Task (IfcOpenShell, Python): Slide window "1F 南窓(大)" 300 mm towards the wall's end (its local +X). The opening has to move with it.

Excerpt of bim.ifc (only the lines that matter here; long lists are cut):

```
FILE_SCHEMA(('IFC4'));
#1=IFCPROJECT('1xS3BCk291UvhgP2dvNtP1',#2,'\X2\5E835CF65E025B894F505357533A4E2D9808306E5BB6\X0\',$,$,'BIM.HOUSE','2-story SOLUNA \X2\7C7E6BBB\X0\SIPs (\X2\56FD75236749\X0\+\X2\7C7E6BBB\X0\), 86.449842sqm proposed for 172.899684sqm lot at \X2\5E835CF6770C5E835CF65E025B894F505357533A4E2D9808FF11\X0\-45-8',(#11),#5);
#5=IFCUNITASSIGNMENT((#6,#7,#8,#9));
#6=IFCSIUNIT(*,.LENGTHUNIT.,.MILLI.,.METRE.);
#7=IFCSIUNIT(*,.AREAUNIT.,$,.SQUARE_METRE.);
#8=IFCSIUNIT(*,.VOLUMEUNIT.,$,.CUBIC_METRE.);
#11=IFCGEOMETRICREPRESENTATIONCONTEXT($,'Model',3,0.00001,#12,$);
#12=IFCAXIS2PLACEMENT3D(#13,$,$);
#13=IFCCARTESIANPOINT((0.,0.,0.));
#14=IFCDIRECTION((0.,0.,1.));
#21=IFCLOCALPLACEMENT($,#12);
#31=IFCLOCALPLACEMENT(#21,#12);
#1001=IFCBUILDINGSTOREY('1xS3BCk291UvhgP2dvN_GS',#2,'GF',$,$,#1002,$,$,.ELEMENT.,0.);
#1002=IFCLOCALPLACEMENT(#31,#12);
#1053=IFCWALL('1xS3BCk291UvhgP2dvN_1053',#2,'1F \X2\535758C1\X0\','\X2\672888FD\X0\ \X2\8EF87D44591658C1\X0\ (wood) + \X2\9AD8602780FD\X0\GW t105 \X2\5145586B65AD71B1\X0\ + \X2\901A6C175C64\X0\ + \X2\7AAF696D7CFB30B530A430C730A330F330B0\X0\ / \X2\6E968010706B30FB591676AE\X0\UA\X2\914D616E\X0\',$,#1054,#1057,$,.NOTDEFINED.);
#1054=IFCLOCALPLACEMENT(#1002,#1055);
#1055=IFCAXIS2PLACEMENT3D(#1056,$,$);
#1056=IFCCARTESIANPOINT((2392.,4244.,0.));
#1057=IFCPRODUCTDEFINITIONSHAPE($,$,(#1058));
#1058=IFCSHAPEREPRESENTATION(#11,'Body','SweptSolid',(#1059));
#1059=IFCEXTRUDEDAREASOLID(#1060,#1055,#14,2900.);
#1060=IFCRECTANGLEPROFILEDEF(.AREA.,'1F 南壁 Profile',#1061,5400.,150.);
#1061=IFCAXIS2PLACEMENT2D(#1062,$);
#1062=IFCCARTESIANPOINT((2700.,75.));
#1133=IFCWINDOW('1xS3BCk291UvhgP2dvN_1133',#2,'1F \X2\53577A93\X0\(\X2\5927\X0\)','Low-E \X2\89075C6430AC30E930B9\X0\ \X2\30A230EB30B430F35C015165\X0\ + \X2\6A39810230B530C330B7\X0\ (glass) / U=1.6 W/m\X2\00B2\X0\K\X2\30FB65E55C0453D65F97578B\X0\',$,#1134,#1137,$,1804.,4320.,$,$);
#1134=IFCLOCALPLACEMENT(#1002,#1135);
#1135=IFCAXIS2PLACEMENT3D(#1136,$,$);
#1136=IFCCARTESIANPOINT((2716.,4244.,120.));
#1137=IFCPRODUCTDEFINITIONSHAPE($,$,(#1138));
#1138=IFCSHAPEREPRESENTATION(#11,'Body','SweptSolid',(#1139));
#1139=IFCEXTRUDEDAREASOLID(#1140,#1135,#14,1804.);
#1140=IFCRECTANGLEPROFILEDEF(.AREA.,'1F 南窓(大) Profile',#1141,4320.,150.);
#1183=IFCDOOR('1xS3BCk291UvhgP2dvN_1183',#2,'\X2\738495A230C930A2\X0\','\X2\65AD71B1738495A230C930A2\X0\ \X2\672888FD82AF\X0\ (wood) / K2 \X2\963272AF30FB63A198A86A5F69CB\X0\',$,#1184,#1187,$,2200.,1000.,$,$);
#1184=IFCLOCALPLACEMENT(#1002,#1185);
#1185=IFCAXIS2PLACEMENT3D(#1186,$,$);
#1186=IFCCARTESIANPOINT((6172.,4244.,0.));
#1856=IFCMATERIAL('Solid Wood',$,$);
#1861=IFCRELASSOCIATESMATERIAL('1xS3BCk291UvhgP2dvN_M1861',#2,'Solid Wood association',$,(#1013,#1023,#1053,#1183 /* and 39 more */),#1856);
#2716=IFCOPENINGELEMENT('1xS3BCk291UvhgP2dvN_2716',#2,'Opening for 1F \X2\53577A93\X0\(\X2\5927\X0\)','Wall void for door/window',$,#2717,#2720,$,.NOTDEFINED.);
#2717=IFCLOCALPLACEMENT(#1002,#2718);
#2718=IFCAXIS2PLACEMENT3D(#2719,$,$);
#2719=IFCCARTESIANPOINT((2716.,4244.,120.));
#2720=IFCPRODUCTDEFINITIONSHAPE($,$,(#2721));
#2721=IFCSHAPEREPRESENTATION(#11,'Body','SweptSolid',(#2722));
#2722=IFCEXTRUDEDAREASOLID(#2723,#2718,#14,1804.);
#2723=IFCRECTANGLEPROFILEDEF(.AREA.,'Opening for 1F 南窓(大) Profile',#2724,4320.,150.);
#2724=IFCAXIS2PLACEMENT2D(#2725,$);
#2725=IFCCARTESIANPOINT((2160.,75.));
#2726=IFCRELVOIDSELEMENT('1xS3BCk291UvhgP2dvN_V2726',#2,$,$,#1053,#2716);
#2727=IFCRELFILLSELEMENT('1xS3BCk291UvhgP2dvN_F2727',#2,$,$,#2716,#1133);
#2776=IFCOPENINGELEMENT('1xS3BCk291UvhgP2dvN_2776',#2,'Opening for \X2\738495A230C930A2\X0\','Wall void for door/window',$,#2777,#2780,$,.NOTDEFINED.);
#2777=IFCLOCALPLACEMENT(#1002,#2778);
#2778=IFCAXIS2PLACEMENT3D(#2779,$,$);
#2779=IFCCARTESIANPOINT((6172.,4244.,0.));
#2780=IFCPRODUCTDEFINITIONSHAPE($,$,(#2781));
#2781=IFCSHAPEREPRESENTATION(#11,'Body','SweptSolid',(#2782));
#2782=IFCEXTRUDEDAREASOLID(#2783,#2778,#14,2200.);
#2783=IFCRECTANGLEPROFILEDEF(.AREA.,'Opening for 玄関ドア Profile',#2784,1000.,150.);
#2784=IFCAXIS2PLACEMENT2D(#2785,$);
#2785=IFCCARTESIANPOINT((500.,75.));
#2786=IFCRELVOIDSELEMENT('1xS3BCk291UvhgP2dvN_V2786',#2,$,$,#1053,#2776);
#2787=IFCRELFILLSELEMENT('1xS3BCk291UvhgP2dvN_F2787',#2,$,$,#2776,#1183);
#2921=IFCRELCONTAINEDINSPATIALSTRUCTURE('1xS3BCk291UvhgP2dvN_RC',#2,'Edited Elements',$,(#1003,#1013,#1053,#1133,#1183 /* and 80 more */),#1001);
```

```python
import ifcopenshell
import ifcopenshell.api.geometry
import ifcopenshell.util.placement
import ifcopenshell.util.unit

model = ifcopenshell.open("bim.ifc")
unit_scale = ifcopenshell.util.unit.calculate_unit_scale(model)

window = model.by_id(1133)
opening = window.FillsVoids[0].RelatingOpeningElement
wall = opening.VoidsElements[0].RelatingBuildingElement

wall_matrix = ifcopenshell.util.placement.get_local_placement(wall.ObjectPlacement)
shift = wall_matrix[:3, 0] * 0.3 / unit_scale
before = ifcopenshell.util.placement.get_local_placement(window.ObjectPlacement)[:3, 3].copy()

# The window is not placed relative to its opening, so move both.
for product in (opening, window):
    matrix = ifcopenshell.util.placement.get_local_placement(product.ObjectPlacement)
    matrix[:3, 3] += shift
    ifcopenshell.api.geometry.edit_object_placement(model, product=product, matrix=matrix, is_si=False)

after = ifcopenshell.util.placement.get_local_placement(window.ObjectPlacement)[:3, 3]
print("window moved by", (after - before).round(3) + 0.0)

model.write("bim_v2.ifc")
```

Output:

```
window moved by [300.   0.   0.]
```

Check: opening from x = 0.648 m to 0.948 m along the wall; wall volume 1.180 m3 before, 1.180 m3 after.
